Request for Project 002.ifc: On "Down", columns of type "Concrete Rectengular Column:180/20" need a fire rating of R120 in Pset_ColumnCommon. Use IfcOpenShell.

First a look at what the model holds.

```python
import ifcopenshell
import ifcopenshell.util.element

model = ifcopenshell.open("Project 002.ifc")
print(model.schema)
storey = next(s for s in model.by_type("IfcBuildingStorey") if s.Name == "Down")
columns = [e for e in ifcopenshell.util.element.get_decomposition(storey) if e.is_a("IfcColumn")]
seen = {}
for e in columns:
    element_type = ifcopenshell.util.element.get_type(e)
    key = (element_type.Name if element_type != e and element_type else None, ifcopenshell.util.element.get_pset(e, "Pset_ColumnCommon", "FireRating"))
    seen[key] = seen.get(key, 0) + 1
for (name, value), count in sorted(seen.items(), key=str):
    print(count, "x", name, "|", value)
```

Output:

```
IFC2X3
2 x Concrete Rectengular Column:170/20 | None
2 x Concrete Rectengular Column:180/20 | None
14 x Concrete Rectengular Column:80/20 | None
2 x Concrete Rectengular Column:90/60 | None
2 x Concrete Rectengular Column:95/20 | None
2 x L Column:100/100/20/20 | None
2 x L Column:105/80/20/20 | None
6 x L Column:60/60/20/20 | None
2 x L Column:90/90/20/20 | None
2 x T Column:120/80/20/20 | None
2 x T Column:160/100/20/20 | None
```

```python
import ifcopenshell
import ifcopenshell.api.pset
import ifcopenshell.util.element

model = ifcopenshell.open("Project 002.ifc")

storey = next(s for s in model.by_type("IfcBuildingStorey") if s.Name == "Down")
columns = [e for e in ifcopenshell.util.element.get_decomposition(storey) if e.is_a("IfcColumn")]

count = 0
for e in columns:
    element_type = ifcopenshell.util.element.get_type(e)
    if element_type in (None, e) or element_type.Name != "Concrete Rectengular Column:180/20":
        continue
    # add_pset returns the element's existing set when there is one.
    pset = ifcopenshell.api.pset.add_pset(model, product=e, name="Pset_ColumnCommon")
    ifcopenshell.api.pset.edit_pset(model, pset=pset, properties={"FireRating": "R120"})
    count += 1

print(count, "columns updated")

model.write("Project 002-out.ifc")
```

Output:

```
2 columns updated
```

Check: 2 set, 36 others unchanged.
